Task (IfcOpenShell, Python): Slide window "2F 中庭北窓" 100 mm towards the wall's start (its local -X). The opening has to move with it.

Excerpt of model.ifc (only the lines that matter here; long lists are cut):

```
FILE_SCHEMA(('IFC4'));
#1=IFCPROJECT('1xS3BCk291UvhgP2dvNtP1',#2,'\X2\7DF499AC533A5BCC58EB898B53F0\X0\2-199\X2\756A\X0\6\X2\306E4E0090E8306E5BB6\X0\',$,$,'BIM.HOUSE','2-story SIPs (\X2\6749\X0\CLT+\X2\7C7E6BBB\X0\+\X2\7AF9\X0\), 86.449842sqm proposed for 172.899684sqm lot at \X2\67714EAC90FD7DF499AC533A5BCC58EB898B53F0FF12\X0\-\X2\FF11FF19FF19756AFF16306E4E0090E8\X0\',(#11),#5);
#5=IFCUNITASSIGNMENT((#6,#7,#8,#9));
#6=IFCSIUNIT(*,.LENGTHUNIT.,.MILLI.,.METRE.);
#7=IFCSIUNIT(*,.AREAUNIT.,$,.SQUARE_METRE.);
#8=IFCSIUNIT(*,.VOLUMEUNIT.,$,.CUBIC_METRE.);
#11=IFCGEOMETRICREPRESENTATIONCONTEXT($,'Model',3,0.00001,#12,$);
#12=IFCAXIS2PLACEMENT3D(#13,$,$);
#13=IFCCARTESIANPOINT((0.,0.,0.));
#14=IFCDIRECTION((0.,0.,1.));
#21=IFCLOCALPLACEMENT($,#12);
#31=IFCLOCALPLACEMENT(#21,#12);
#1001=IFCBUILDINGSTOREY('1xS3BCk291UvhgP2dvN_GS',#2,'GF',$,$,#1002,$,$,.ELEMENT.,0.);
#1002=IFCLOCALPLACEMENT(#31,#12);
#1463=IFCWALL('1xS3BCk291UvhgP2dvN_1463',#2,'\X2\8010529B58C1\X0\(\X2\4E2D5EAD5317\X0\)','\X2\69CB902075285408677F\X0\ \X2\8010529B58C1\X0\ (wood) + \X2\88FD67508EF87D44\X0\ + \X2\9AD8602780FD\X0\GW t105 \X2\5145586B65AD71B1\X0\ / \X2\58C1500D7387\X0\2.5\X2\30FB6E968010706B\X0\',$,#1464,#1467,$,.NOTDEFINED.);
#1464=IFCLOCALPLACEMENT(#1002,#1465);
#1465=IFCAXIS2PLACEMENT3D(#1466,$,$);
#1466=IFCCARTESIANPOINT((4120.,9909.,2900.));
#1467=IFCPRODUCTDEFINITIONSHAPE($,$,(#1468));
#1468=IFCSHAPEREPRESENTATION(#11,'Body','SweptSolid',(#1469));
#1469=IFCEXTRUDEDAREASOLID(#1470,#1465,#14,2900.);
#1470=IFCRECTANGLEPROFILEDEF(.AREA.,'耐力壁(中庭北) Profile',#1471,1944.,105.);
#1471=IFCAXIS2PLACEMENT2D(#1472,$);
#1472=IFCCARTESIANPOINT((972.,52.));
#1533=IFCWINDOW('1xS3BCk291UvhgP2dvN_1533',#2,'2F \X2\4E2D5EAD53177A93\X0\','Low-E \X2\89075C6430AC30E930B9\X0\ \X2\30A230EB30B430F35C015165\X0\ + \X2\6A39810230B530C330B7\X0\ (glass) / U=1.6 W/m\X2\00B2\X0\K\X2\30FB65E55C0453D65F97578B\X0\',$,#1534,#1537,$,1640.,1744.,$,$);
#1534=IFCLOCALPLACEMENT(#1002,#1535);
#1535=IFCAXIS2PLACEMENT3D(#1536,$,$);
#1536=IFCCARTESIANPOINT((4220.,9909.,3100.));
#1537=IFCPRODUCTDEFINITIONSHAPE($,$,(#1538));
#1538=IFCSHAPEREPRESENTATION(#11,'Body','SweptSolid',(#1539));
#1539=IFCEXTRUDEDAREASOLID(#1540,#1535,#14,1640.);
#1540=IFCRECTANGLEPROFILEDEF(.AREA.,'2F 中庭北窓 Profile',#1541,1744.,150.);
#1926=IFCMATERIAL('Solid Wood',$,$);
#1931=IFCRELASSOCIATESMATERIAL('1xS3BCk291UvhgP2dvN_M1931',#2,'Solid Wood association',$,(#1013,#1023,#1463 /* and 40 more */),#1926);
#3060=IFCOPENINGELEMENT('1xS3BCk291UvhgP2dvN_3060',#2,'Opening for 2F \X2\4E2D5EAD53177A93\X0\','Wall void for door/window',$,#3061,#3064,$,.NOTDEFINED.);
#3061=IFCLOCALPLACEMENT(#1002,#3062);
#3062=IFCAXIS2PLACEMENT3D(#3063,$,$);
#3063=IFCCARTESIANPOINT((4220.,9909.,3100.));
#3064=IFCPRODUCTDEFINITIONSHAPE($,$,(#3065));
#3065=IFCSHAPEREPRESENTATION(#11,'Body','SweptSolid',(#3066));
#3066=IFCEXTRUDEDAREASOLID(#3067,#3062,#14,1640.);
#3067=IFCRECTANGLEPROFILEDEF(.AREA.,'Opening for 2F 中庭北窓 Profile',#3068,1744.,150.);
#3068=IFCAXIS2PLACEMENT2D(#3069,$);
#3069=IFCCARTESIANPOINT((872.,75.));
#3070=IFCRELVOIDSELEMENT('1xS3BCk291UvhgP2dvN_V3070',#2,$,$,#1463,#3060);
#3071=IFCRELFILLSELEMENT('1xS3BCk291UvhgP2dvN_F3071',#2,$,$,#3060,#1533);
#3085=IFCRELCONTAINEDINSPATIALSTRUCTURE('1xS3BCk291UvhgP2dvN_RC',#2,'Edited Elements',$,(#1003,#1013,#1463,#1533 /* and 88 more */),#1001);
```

```python
import ifcopenshell
import ifcopenshell.api.geometry
import ifcopenshell.util.placement
import ifcopenshell.util.unit

model = ifcopenshell.open("model.ifc")
unit_scale = ifcopenshell.util.unit.calculate_unit_scale(model)

window = model.by_guid("1xS3BCk291UvhgP2dvN_1533")
opening = window.FillsVoids[0].RelatingOpeningElement
wall = opening.VoidsElements[0].RelatingBuildingElement

wall_matrix = ifcopenshell.util.placement.get_local_placement(wall.ObjectPlacement)
shift = wall_matrix[:3, 0] * -0.1 / unit_scale
before = ifcopenshell.util.placement.get_local_placement(window.ObjectPlacement)[:3, 3].copy()

# The window is not placed relative to its opening, so move both.
for product in (opening, window):
    matrix = ifcopenshell.util.placement.get_local_placement(product.ObjectPlacement)
    matrix[:3, 3] += shift
    ifcopenshell.api.geometry.edit_object_placement(model, product=product, matrix=matrix, is_si=False)

after = ifcopenshell.util.placement.get_local_placement(window.ObjectPlacement)[:3, 3]
print("window moved by", (after - before).round(3) + 0.0)

model.write("model_updated.ifc")
```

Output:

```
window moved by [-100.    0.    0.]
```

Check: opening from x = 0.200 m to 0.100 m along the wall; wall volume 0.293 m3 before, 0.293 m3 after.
